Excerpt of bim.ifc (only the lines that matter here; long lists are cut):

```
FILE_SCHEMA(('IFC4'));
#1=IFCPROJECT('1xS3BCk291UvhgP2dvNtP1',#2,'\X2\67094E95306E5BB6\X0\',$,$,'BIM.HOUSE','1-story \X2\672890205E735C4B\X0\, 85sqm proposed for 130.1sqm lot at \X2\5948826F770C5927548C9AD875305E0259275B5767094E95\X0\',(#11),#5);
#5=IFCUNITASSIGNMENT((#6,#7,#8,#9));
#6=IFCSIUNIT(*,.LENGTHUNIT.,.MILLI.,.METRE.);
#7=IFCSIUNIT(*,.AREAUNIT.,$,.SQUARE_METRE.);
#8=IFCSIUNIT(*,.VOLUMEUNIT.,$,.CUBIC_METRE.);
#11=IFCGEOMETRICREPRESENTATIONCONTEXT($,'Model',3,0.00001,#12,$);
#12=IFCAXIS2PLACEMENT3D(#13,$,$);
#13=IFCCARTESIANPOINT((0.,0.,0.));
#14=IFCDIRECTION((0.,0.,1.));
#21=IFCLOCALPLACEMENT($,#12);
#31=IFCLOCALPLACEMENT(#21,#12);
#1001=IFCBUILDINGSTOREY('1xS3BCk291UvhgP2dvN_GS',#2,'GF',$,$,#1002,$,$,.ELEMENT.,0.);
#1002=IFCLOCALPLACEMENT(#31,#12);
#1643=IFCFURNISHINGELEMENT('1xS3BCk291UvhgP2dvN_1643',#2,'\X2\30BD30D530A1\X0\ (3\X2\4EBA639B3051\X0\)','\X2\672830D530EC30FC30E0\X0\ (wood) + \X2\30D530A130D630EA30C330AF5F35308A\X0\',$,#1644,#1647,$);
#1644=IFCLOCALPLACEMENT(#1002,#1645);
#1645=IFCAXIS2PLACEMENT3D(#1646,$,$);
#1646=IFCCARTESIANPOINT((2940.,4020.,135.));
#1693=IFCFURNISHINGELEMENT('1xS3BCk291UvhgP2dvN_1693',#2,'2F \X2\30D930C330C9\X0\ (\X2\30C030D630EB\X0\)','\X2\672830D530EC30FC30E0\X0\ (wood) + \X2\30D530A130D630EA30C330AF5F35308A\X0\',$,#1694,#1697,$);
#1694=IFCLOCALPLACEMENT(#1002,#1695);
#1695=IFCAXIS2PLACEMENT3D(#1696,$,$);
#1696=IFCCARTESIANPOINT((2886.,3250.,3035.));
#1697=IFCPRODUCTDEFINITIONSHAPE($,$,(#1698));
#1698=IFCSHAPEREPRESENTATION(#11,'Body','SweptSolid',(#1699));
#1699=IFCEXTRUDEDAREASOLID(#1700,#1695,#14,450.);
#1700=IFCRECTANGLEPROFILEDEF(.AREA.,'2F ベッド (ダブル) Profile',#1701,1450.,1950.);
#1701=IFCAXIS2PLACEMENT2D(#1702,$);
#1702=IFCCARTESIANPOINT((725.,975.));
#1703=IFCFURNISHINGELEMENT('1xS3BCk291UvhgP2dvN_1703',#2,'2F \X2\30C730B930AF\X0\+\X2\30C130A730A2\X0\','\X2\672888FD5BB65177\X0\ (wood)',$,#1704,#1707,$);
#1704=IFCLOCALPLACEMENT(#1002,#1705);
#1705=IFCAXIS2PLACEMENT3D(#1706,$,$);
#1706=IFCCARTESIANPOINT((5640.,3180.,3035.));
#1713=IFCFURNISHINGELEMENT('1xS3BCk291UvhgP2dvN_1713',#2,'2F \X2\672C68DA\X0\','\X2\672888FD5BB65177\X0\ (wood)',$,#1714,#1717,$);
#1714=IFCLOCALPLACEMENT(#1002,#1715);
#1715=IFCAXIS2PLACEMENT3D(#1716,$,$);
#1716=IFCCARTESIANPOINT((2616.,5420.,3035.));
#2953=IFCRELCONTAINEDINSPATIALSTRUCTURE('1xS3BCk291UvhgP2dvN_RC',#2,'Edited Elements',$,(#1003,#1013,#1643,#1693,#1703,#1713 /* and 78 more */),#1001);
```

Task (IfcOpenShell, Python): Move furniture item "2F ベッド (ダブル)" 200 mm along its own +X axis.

```python
import ifcopenshell
import ifcopenshell.api.geometry
import ifcopenshell.util.placement
import ifcopenshell.util.unit

model = ifcopenshell.open("bim.ifc")
unit_scale = ifcopenshell.util.unit.calculate_unit_scale(model)

item = model.by_guid("1xS3BCk291UvhgP2dvN_1693")
matrix = ifcopenshell.util.placement.get_local_placement(item.ObjectPlacement)
matrix[:3, 3] += matrix[:3, 0] * 0.2 / unit_scale
ifcopenshell.api.geometry.edit_object_placement(model, product=item, matrix=matrix, is_si=False)

print(ifcopenshell.util.placement.get_local_placement(item.ObjectPlacement).round(3) + 0.0)

model.write("bim_updated.ifc")
```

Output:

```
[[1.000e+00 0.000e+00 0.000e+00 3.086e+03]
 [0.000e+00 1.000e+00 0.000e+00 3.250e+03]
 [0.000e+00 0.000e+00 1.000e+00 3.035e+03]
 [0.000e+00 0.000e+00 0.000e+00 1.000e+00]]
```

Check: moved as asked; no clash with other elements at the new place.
